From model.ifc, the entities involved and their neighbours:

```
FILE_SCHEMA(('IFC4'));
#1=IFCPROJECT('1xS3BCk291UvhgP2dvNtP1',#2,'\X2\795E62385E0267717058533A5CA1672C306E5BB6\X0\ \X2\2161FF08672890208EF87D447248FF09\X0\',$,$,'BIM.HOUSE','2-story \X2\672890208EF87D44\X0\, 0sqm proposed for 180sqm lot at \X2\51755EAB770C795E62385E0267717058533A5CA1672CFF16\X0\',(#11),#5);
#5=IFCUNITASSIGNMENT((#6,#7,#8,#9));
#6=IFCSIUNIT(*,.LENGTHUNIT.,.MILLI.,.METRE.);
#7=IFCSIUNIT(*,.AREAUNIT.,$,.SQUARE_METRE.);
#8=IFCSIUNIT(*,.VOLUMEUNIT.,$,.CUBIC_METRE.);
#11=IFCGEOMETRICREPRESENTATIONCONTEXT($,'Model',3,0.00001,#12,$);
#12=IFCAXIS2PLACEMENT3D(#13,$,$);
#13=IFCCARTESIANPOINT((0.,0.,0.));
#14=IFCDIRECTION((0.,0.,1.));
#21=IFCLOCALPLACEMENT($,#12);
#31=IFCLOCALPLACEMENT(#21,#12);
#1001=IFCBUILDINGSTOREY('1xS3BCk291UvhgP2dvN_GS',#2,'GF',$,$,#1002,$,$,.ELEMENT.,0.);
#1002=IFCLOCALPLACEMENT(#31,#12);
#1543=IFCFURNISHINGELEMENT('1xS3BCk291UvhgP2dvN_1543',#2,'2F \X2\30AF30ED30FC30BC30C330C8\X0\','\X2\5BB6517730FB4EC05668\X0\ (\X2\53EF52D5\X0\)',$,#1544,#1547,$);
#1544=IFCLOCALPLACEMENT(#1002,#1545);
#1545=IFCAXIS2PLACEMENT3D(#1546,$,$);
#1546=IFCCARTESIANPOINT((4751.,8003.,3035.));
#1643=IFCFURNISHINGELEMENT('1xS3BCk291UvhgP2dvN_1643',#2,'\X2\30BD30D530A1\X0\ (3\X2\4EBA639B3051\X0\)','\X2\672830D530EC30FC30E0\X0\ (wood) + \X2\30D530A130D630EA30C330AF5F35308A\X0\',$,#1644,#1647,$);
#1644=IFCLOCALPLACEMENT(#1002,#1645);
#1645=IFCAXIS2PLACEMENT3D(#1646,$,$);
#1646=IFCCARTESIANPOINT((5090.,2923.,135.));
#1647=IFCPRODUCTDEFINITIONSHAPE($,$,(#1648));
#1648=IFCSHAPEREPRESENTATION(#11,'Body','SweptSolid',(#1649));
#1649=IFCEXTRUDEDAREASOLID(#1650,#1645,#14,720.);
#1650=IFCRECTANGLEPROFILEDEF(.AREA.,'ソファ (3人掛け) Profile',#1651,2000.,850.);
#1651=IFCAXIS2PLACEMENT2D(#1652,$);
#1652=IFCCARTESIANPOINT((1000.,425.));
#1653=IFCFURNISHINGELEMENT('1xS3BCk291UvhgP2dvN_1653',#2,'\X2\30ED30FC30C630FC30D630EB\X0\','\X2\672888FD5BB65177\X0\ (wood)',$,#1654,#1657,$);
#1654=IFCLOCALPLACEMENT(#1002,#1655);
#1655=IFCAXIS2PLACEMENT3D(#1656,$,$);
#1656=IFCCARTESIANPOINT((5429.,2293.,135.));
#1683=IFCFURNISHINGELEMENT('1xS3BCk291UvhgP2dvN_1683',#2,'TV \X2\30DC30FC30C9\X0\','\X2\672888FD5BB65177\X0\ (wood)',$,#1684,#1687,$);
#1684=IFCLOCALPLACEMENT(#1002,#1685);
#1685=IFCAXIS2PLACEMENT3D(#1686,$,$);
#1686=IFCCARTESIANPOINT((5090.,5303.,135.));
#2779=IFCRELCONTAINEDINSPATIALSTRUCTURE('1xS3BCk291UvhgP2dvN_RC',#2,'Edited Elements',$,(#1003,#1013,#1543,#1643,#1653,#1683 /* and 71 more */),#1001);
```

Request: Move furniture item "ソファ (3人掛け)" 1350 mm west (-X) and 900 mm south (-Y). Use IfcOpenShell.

```python
import ifcopenshell
import ifcopenshell.api.geometry
import ifcopenshell.util.placement

model = ifcopenshell.open("model.ifc")

item = model.by_guid("1xS3BCk291UvhgP2dvN_1643")
matrix = ifcopenshell.util.placement.get_local_placement(item.ObjectPlacement)
matrix[0, 3] -= 1350.0
matrix[1, 3] -= 900.0
ifcopenshell.api.geometry.edit_object_placement(model, product=item, matrix=matrix, is_si=False)

print(ifcopenshell.util.placement.get_local_placement(item.ObjectPlacement).round(3) + 0.0)

model.write("model-out.ifc")
```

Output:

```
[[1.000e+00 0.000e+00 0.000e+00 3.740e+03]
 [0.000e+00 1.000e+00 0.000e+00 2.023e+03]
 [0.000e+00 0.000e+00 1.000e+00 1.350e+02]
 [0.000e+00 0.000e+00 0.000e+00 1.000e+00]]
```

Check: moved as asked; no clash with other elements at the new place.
